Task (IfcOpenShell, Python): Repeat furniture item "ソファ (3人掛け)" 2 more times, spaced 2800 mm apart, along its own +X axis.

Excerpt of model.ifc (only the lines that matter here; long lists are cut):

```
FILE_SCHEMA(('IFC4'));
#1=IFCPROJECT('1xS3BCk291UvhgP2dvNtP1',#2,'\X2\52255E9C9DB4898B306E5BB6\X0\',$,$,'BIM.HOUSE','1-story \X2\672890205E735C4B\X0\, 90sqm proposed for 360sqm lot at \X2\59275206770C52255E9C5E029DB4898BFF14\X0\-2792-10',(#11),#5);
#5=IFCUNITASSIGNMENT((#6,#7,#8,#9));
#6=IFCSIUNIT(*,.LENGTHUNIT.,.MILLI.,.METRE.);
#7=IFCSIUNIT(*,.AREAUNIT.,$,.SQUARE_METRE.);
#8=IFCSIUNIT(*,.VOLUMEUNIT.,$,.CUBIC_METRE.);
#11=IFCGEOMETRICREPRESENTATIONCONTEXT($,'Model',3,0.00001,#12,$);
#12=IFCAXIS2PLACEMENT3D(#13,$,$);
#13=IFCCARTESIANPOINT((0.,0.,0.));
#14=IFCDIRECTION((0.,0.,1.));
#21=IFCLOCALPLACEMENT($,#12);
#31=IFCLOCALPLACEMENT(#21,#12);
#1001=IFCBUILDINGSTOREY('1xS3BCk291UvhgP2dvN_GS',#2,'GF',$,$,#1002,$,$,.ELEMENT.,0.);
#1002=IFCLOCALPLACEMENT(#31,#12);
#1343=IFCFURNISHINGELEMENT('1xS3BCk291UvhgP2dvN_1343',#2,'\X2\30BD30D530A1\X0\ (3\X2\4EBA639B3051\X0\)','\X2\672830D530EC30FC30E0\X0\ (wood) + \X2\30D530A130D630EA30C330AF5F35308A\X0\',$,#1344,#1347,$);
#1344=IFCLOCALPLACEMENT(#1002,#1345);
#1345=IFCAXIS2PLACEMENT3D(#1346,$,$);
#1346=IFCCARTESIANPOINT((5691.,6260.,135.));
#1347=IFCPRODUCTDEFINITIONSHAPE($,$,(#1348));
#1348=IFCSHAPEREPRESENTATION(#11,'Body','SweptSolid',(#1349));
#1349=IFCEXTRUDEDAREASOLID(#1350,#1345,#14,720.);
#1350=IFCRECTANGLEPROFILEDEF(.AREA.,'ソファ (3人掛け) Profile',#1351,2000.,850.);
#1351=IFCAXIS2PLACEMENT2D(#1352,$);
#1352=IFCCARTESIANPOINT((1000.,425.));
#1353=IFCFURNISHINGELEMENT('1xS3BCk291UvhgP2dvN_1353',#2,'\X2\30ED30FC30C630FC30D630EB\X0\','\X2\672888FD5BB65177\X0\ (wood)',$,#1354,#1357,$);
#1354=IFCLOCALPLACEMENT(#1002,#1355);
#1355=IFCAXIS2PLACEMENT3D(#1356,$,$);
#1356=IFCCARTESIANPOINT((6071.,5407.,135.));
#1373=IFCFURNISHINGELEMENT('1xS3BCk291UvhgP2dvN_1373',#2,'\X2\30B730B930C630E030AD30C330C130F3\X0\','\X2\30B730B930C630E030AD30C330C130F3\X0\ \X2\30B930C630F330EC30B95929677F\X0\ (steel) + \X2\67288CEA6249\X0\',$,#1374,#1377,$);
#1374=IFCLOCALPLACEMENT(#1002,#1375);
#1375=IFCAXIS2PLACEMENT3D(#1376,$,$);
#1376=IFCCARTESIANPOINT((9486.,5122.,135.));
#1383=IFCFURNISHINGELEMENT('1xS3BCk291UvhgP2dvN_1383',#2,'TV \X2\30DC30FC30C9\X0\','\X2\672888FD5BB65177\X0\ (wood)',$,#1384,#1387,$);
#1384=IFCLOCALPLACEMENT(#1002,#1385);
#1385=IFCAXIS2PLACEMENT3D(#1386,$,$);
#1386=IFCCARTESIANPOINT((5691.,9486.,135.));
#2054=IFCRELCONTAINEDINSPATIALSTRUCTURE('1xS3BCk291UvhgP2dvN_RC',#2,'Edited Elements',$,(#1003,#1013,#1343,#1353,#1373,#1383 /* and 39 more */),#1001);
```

```python
import ifcopenshell
import ifcopenshell.api.geometry
import ifcopenshell.api.root
import ifcopenshell.util.element
import ifcopenshell.util.placement
import ifcopenshell.util.unit

model = ifcopenshell.open("model.ifc")
unit_scale = ifcopenshell.util.unit.calculate_unit_scale(model)


def reuse_history(source, copy):
    """copy_class also copies each property set's owner history, people and application; keep the originals."""
    for rel in copy.IsDefinedBy:
        if rel.is_a("IfcRelDefinesByProperties") and (history := rel.RelatingPropertyDefinition.OwnerHistory):
            rel.RelatingPropertyDefinition.OwnerHistory = source.OwnerHistory
            ifcopenshell.util.element.remove_deep2(model, history)


source = model.by_id(1343)
base = ifcopenshell.util.placement.get_local_placement(source.ObjectPlacement)
step = base[:3, 0] * 2.8 / unit_scale

for i in range(1, 3):
    copy = ifcopenshell.api.root.copy_class(model, product=source)
    copy.Representation = ifcopenshell.util.element.copy_deep(
        model, source.Representation, exclude=["IfcGeometricRepresentationContext", "IfcRepresentationMap"]
    )
    reuse_history(source, copy)
    matrix = base.copy()
    matrix[:3, 3] += i * step
    print("added at", matrix[:3, 3].round(3) + 0.0)
    ifcopenshell.api.geometry.edit_object_placement(model, product=copy, matrix=matrix, is_si=False)

model.write("model_rev.ifc")
```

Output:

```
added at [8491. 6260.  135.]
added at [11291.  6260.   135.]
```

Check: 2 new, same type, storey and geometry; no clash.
